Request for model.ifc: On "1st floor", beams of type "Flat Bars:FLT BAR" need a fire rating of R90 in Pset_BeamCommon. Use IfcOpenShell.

First a look at what the model holds.

```python
import ifcopenshell
import ifcopenshell.util.element

model = ifcopenshell.open("model.ifc")
print(model.schema)
storey = next(s for s in model.by_type("IfcBuildingStorey") if s.Name == "1st floor")
beams = [e for e in ifcopenshell.util.element.get_decomposition(storey) if e.is_a("IfcBeam")]
seen = {}
for e in beams:
    element_type = ifcopenshell.util.element.get_type(e)
    key = (element_type.Name if element_type != e and element_type else None, ifcopenshell.util.element.get_pset(e, "Pset_BeamCommon", "FireRating"))
    seen[key] = seen.get(key, 0) + 1
for (name, value), count in sorted(seen.items(), key=str):
    print(count, "x", name, "|", value)
```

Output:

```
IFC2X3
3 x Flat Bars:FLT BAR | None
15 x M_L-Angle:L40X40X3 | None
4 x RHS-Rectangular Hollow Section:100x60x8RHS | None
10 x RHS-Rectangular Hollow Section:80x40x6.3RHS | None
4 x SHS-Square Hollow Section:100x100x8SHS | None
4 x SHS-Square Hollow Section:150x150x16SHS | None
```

```python
import ifcopenshell
import ifcopenshell.api.pset
import ifcopenshell.util.element

model = ifcopenshell.open("model.ifc")

storey = next(s for s in model.by_type("IfcBuildingStorey") if s.Name == "1st floor")
beams = [e for e in ifcopenshell.util.element.get_decomposition(storey) if e.is_a("IfcBeam")]

count = 0
for e in beams:
    element_type = ifcopenshell.util.element.get_type(e)
    if element_type in (None, e) or element_type.Name != "Flat Bars:FLT BAR":
        continue
    # add_pset returns the element's existing set when there is one.
    pset = ifcopenshell.api.pset.add_pset(model, product=e, name="Pset_BeamCommon")
    ifcopenshell.api.pset.edit_pset(model, pset=pset, properties={"FireRating": "R90"})
    count += 1

print(count, "beams updated")

model.write("model_v2.ifc")
```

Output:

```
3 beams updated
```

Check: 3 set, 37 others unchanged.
